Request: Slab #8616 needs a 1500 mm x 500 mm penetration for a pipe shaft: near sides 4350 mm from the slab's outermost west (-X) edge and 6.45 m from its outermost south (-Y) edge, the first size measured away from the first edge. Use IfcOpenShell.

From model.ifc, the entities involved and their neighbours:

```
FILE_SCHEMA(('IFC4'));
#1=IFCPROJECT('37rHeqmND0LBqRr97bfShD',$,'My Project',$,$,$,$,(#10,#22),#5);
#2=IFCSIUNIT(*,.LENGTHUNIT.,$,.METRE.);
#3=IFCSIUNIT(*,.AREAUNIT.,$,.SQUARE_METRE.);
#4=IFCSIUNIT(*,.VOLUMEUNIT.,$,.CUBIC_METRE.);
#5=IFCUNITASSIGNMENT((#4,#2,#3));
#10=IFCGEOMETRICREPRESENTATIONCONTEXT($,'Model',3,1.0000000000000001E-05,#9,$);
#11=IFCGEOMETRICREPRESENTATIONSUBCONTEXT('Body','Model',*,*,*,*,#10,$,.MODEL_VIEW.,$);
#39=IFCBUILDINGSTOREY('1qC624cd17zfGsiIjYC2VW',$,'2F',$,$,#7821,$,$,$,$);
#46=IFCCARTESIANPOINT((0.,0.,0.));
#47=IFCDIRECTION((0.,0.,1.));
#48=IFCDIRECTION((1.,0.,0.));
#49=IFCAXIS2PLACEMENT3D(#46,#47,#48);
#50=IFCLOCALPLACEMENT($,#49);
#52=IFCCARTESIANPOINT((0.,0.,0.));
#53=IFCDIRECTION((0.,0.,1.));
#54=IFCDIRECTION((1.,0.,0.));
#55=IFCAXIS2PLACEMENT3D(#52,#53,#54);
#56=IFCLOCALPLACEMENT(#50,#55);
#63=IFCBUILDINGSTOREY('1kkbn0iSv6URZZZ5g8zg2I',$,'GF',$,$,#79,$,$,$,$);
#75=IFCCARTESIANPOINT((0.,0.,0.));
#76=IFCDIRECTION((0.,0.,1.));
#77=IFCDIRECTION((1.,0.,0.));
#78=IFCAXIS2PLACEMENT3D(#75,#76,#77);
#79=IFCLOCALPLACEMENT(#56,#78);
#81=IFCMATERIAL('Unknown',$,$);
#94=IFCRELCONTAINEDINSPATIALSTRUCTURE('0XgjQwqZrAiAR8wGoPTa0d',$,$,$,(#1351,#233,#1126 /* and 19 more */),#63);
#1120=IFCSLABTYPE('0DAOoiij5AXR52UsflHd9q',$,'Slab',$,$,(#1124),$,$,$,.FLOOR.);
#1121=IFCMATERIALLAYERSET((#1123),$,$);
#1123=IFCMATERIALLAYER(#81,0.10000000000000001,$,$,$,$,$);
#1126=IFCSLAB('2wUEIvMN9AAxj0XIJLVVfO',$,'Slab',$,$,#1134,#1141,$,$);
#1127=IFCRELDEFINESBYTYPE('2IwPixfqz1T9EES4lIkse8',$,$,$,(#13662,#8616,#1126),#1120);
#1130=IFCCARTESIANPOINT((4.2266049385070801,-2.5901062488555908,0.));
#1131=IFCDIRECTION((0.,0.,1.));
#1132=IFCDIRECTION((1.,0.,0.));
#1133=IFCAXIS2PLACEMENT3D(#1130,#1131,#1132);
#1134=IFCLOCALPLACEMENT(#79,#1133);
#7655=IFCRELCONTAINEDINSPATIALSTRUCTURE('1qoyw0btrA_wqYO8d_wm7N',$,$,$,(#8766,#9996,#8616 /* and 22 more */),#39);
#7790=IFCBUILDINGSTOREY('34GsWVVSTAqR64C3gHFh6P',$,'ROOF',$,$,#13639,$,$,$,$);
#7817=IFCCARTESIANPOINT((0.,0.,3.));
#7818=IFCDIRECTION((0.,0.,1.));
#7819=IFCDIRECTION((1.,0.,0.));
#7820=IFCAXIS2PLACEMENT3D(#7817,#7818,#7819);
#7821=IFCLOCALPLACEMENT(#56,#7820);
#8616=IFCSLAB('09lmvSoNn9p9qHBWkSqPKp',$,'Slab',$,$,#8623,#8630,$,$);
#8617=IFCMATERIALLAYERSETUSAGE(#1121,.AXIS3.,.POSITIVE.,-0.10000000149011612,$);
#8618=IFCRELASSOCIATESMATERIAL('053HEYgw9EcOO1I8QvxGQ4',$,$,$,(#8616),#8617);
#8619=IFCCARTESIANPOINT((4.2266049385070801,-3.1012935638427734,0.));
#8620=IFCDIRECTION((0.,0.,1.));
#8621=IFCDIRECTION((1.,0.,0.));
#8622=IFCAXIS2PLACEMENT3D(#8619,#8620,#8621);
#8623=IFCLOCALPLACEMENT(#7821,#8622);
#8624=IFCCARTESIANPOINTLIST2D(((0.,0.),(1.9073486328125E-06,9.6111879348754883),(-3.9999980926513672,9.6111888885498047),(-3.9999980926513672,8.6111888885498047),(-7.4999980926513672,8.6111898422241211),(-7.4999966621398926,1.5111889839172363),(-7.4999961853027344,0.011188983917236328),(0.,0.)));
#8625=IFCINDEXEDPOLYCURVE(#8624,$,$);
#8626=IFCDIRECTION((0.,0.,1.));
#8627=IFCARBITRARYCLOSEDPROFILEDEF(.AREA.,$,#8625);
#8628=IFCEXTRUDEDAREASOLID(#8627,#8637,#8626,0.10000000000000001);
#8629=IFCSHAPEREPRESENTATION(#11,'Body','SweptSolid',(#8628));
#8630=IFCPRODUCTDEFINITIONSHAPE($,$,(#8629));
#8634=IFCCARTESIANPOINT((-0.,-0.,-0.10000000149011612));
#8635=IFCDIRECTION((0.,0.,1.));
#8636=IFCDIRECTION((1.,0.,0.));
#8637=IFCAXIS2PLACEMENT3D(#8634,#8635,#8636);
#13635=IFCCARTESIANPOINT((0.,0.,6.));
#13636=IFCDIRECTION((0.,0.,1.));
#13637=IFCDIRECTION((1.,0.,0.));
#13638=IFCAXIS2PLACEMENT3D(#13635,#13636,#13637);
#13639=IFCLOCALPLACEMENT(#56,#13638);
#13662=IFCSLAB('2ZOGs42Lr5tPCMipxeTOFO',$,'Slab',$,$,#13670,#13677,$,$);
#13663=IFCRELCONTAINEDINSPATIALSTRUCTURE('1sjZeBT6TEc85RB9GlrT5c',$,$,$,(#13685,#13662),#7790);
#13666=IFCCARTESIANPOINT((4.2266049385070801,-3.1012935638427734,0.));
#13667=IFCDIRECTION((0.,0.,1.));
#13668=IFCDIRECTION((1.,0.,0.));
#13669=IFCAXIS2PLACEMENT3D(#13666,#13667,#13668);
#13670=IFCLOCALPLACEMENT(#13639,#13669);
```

```python
import numpy as np
import ifcopenshell
import ifcopenshell.api.feature
import ifcopenshell.api.geometry
import ifcopenshell.api.root
import ifcopenshell.geom
import ifcopenshell.util.placement
import ifcopenshell.util.representation
import ifcopenshell.util.shape
import ifcopenshell.util.unit

model = ifcopenshell.open("model.ifc")
unit_scale = ifcopenshell.util.unit.calculate_unit_scale(model)
settings = ifcopenshell.geom.settings()


def volume(element):
    """Net volume in cubic metres, openings subtracted."""
    shape = ifcopenshell.geom.create_shape(settings, element)
    return ifcopenshell.util.shape.get_volume(shape.geometry)


slab = model.by_guid("09lmvSoNn9p9qHBWkSqPKp")
before = volume(slab)

# Extent in the slab's own axes, in metres. The edges named are its -X and -Y sides.
slab_shape = ifcopenshell.geom.create_shape(settings, slab)
vertices = ifcopenshell.util.shape.get_vertices(slab_shape.geometry)
x_min, y_min, bottom = vertices.min(axis=0)
top = vertices[:, 2].max()

opening = ifcopenshell.api.root.create_entity(model, ifc_class="IfcOpeningElement", name="Pipe shaft opening", predefined_type="OPENING")
context = ifcopenshell.util.representation.get_context(model, "Model", "Body", "MODEL_VIEW")
width, depth = 1.5, 0.5
outline = [(0.0, 0.0), (width, 0.0), (width, depth), (0.0, depth), (0.0, 0.0)]
# Overshoot both faces by 50 mm so the cut is clean.
shape = ifcopenshell.api.geometry.add_slab_representation(
    model, context=context, depth=top - bottom + 0.1, polyline=outline
)
ifcopenshell.api.geometry.assign_representation(model, product=opening, representation=shape)

matrix = ifcopenshell.util.placement.get_local_placement(slab.ObjectPlacement)
matrix[:, 3] = matrix @ np.append(np.array([x_min + 4.35, y_min + 6.45, bottom - 0.05]) / unit_scale, 1.0)
ifcopenshell.api.geometry.edit_object_placement(model, product=opening, matrix=matrix, is_si=False)
ifcopenshell.api.feature.add_feature(model, feature=opening, element=slab)

after = volume(slab)

print(f"slab volume {before:.3f} -> {after:.3f} m3")

model.write("model_updated.ifc")
```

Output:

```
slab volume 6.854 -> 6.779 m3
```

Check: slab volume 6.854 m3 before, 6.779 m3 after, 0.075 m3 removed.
